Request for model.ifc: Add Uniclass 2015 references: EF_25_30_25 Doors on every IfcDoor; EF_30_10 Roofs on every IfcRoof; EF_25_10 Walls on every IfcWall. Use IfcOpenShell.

First a look at what the model holds.

```python
import ifcopenshell

model = ifcopenshell.open("model.ifc")
print(model.schema)
print("classifications:", [c.Name for c in model.by_type("IfcClassification")])
for ifc_class in ("IfcDoor", "IfcRoof", "IfcStair", "IfcWall", "IfcWindow"):
    print(ifc_class, len(model.by_type(ifc_class)))
```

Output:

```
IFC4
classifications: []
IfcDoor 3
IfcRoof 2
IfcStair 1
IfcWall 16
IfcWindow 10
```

```python
import ifcopenshell
import ifcopenshell.api.classification

model = ifcopenshell.open("model.ifc")

system = ifcopenshell.api.classification.add_classification(model, classification="Uniclass 2015")

codes = {
    "IfcDoor": ("EF_25_30_25", "Doors"),
    "IfcRoof": ("EF_30_10", "Roofs"),
    "IfcWall": ("EF_25_10", "Walls"),
}
for ifc_class, (code, name) in codes.items():
    products = model.by_type(ifc_class)
    ifcopenshell.api.classification.add_reference(
        model, products=products, classification=system, identification=code, name=name
    )
    print(code, len(products))

model.write("model_rev.ifc")
```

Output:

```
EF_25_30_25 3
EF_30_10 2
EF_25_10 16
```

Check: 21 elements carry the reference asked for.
